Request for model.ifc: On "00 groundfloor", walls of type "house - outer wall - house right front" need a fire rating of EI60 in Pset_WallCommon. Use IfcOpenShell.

First a look at what the model holds.

```python
import ifcopenshell
import ifcopenshell.util.element

model = ifcopenshell.open("model.ifc")
print(model.schema)
storey = next(s for s in model.by_type("IfcBuildingStorey") if s.Name == "00 groundfloor")
walls = [e for e in ifcopenshell.util.element.get_decomposition(storey) if e.is_a("IfcWall")]
seen = {}
for e in walls:
    element_type = ifcopenshell.util.element.get_type(e)
    key = (element_type.Name if element_type != e and element_type else None, ifcopenshell.util.element.get_pset(e, "Pset_WallCommon", "FireRating"))
    seen[key] = seen.get(key, 0) + 1
for (name, value), count in sorted(seen.items(), key=str):
    print(count, "x", name, "|", value)
```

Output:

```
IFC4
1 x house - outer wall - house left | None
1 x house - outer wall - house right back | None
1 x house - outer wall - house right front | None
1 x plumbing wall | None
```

```python
import ifcopenshell
import ifcopenshell.api.pset
import ifcopenshell.util.element

model = ifcopenshell.open("model.ifc")

storey = next(s for s in model.by_type("IfcBuildingStorey") if s.Name == "00 groundfloor")
walls = [e for e in ifcopenshell.util.element.get_decomposition(storey) if e.is_a("IfcWall")]

count = 0
for e in walls:
    element_type = ifcopenshell.util.element.get_type(e)
    if element_type in (None, e) or element_type.Name != "house - outer wall - house right front":
        continue
    # add_pset returns the element's existing set when there is one.
    pset = ifcopenshell.api.pset.add_pset(model, product=e, name="Pset_WallCommon")
    ifcopenshell.api.pset.edit_pset(model, pset=pset, properties={"FireRating": "EI60"})
    count += 1

print(count, "walls updated")

model.write("model-out.ifc")
```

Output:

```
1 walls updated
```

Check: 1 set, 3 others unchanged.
